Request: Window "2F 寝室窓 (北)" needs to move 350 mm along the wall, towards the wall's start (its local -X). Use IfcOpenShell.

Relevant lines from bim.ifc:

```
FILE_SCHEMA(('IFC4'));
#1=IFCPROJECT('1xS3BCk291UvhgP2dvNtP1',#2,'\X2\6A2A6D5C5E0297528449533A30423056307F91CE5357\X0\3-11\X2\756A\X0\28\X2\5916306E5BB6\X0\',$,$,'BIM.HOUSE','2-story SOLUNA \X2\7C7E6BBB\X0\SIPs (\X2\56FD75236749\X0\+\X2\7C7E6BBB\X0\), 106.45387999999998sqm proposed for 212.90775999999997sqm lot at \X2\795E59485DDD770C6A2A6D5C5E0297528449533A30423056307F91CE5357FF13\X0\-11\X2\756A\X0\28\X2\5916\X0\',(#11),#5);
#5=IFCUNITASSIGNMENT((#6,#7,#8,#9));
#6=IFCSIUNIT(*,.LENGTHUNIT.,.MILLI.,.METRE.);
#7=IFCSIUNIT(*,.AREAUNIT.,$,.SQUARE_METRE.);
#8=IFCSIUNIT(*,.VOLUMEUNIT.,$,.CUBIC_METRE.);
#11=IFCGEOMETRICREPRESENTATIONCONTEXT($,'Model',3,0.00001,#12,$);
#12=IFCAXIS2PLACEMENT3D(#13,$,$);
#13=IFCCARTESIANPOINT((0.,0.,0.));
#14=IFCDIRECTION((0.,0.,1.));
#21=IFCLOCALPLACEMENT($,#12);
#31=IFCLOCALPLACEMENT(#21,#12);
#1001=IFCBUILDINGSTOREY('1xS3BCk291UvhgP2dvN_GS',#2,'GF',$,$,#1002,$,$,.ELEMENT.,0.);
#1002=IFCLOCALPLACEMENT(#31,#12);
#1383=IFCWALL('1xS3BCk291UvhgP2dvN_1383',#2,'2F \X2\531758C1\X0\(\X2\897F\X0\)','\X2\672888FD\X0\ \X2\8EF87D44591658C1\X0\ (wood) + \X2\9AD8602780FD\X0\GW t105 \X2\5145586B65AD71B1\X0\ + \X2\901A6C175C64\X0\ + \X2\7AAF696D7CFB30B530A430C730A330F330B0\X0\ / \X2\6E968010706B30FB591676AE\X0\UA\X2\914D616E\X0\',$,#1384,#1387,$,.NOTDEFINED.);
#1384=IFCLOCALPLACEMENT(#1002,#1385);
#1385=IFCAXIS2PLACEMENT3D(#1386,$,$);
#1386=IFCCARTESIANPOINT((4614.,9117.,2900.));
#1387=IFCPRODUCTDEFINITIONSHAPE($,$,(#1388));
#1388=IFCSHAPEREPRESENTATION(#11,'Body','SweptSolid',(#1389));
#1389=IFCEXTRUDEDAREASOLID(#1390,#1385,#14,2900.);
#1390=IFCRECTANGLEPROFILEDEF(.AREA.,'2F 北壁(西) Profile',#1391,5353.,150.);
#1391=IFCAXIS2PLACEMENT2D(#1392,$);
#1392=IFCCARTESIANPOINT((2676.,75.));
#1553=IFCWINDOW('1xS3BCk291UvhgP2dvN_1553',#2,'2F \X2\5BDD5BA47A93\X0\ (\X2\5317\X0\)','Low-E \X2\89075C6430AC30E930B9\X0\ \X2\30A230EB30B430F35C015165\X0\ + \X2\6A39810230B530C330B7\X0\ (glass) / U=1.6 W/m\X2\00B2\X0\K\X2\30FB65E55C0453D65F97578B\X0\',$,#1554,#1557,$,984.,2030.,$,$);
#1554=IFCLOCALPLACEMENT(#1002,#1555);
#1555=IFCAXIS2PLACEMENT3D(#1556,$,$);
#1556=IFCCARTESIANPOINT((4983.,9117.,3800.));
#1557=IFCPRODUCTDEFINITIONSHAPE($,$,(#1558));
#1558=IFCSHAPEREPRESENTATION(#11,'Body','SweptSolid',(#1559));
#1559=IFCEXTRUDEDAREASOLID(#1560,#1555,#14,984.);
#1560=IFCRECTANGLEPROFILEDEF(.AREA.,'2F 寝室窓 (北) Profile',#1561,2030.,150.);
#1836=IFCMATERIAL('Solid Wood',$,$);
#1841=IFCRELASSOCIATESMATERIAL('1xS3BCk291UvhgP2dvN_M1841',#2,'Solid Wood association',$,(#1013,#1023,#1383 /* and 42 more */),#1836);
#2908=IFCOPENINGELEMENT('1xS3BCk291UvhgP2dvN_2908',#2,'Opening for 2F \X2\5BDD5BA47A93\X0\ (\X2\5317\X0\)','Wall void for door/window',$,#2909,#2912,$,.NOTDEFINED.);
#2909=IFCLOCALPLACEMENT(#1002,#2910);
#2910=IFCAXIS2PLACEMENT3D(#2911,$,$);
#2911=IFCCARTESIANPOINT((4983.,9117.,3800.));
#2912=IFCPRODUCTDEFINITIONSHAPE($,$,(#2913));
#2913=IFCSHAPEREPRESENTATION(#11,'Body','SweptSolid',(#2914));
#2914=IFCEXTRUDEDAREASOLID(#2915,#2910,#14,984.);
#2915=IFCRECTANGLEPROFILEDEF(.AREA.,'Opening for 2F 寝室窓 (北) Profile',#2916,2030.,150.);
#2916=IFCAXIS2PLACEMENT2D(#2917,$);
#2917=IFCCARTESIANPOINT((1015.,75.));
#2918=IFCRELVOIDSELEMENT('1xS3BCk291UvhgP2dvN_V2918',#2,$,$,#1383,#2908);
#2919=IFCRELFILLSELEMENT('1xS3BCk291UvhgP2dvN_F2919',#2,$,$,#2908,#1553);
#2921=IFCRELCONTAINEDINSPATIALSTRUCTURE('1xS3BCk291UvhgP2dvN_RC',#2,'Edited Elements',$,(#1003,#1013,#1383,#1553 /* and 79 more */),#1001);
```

```python
import ifcopenshell
import ifcopenshell.api.geometry
import ifcopenshell.util.placement

model = ifcopenshell.open("bim.ifc")

window = model.by_guid("1xS3BCk291UvhgP2dvN_1553")
opening = window.FillsVoids[0].RelatingOpeningElement
wall = opening.VoidsElements[0].RelatingBuildingElement

wall_matrix = ifcopenshell.util.placement.get_local_placement(wall.ObjectPlacement)
shift = wall_matrix[:3, 0] * -350.0
before = ifcopenshell.util.placement.get_local_placement(window.ObjectPlacement)[:3, 3].copy()

# The window is not placed relative to its opening, so move both.
for product in (opening, window):
    matrix = ifcopenshell.util.placement.get_local_placement(product.ObjectPlacement)
    matrix[:3, 3] += shift
    ifcopenshell.api.geometry.edit_object_placement(model, product=product, matrix=matrix, is_si=False)

after = ifcopenshell.util.placement.get_local_placement(window.ObjectPlacement)[:3, 3]
print("window moved by", (after - before).round(3) + 0.0)

model.write("bim-out.ifc")
```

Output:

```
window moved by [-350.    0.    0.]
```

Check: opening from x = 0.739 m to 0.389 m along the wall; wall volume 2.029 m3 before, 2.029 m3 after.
